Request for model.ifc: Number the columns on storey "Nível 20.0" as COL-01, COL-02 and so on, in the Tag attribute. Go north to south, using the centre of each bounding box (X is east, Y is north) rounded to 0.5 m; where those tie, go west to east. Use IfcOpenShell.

First a look at what the model holds.

```python
import ifcopenshell
import ifcopenshell.util.element
import ifcopenshell.util.placement

model = ifcopenshell.open("model.ifc")
print(model.schema)
storey = next(s for s in model.by_type("IfcBuildingStorey") if s.Name == "Nível 20.0")
columns = [e for e in ifcopenshell.util.element.get_decomposition(storey) if e.is_a("IfcColumn")]
for e in sorted(columns, key=lambda e: e.id()):
    origin = ifcopenshell.util.placement.get_local_placement(e.ObjectPlacement)[:3, 3]
    print(e.id(), e.Tag, e.Name, origin.round(2) + 0.0, sep=" | ")
```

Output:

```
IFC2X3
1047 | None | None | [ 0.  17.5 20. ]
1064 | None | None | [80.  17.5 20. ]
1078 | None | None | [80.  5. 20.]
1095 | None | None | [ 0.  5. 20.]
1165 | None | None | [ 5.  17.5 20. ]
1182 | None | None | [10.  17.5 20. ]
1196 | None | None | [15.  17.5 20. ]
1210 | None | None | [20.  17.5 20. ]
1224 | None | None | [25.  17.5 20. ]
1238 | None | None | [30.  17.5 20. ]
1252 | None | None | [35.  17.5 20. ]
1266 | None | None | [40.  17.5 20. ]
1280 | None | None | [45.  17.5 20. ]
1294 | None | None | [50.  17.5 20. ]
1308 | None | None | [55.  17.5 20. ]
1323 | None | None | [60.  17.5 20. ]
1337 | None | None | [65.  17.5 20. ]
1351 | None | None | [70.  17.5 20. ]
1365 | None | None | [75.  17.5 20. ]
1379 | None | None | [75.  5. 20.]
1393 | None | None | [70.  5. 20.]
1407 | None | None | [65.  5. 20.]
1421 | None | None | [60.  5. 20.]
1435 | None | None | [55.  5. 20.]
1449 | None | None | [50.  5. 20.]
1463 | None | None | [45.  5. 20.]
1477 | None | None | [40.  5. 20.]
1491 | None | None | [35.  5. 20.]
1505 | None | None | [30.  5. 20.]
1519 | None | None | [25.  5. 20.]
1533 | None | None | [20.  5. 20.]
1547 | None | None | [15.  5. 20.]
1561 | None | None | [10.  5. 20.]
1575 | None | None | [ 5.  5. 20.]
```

```python
import ifcopenshell
import ifcopenshell.geom
import ifcopenshell.util.element
import ifcopenshell.util.shape

model = ifcopenshell.open("model.ifc")
settings = ifcopenshell.geom.settings()
settings.set("use-world-coords", True)


def centre(element):
    shape = ifcopenshell.geom.create_shape(settings, element)
    return ifcopenshell.util.shape.get_bbox_centroid(shape.geometry)


storey = next(s for s in model.by_type("IfcBuildingStorey") if s.Name == "Nível 20.0")
columns = [e for e in ifcopenshell.util.element.get_decomposition(storey) if e.is_a("IfcColumn")]

# Insertion points can sit at a corner or the storey origin, so sort by the geometry (in metres).
centres = {e: centre(e) for e in columns}
columns.sort(key=lambda e: (-round(centres[e][1] / 0.5), centres[e][0]))

for i, e in enumerate(columns, start=1):
    number = f"COL-{i:02d}"
    e.Tag = number
    print(e.id(), number)

model.write("model_v2.ifc")
```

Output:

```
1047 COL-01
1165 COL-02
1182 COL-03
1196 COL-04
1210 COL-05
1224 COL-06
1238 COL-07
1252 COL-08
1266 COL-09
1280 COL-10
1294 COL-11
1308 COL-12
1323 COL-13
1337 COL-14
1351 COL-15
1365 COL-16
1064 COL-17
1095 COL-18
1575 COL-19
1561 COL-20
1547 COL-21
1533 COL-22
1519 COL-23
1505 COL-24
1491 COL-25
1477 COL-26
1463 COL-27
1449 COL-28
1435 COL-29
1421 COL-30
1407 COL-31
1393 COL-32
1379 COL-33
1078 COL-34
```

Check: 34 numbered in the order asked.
